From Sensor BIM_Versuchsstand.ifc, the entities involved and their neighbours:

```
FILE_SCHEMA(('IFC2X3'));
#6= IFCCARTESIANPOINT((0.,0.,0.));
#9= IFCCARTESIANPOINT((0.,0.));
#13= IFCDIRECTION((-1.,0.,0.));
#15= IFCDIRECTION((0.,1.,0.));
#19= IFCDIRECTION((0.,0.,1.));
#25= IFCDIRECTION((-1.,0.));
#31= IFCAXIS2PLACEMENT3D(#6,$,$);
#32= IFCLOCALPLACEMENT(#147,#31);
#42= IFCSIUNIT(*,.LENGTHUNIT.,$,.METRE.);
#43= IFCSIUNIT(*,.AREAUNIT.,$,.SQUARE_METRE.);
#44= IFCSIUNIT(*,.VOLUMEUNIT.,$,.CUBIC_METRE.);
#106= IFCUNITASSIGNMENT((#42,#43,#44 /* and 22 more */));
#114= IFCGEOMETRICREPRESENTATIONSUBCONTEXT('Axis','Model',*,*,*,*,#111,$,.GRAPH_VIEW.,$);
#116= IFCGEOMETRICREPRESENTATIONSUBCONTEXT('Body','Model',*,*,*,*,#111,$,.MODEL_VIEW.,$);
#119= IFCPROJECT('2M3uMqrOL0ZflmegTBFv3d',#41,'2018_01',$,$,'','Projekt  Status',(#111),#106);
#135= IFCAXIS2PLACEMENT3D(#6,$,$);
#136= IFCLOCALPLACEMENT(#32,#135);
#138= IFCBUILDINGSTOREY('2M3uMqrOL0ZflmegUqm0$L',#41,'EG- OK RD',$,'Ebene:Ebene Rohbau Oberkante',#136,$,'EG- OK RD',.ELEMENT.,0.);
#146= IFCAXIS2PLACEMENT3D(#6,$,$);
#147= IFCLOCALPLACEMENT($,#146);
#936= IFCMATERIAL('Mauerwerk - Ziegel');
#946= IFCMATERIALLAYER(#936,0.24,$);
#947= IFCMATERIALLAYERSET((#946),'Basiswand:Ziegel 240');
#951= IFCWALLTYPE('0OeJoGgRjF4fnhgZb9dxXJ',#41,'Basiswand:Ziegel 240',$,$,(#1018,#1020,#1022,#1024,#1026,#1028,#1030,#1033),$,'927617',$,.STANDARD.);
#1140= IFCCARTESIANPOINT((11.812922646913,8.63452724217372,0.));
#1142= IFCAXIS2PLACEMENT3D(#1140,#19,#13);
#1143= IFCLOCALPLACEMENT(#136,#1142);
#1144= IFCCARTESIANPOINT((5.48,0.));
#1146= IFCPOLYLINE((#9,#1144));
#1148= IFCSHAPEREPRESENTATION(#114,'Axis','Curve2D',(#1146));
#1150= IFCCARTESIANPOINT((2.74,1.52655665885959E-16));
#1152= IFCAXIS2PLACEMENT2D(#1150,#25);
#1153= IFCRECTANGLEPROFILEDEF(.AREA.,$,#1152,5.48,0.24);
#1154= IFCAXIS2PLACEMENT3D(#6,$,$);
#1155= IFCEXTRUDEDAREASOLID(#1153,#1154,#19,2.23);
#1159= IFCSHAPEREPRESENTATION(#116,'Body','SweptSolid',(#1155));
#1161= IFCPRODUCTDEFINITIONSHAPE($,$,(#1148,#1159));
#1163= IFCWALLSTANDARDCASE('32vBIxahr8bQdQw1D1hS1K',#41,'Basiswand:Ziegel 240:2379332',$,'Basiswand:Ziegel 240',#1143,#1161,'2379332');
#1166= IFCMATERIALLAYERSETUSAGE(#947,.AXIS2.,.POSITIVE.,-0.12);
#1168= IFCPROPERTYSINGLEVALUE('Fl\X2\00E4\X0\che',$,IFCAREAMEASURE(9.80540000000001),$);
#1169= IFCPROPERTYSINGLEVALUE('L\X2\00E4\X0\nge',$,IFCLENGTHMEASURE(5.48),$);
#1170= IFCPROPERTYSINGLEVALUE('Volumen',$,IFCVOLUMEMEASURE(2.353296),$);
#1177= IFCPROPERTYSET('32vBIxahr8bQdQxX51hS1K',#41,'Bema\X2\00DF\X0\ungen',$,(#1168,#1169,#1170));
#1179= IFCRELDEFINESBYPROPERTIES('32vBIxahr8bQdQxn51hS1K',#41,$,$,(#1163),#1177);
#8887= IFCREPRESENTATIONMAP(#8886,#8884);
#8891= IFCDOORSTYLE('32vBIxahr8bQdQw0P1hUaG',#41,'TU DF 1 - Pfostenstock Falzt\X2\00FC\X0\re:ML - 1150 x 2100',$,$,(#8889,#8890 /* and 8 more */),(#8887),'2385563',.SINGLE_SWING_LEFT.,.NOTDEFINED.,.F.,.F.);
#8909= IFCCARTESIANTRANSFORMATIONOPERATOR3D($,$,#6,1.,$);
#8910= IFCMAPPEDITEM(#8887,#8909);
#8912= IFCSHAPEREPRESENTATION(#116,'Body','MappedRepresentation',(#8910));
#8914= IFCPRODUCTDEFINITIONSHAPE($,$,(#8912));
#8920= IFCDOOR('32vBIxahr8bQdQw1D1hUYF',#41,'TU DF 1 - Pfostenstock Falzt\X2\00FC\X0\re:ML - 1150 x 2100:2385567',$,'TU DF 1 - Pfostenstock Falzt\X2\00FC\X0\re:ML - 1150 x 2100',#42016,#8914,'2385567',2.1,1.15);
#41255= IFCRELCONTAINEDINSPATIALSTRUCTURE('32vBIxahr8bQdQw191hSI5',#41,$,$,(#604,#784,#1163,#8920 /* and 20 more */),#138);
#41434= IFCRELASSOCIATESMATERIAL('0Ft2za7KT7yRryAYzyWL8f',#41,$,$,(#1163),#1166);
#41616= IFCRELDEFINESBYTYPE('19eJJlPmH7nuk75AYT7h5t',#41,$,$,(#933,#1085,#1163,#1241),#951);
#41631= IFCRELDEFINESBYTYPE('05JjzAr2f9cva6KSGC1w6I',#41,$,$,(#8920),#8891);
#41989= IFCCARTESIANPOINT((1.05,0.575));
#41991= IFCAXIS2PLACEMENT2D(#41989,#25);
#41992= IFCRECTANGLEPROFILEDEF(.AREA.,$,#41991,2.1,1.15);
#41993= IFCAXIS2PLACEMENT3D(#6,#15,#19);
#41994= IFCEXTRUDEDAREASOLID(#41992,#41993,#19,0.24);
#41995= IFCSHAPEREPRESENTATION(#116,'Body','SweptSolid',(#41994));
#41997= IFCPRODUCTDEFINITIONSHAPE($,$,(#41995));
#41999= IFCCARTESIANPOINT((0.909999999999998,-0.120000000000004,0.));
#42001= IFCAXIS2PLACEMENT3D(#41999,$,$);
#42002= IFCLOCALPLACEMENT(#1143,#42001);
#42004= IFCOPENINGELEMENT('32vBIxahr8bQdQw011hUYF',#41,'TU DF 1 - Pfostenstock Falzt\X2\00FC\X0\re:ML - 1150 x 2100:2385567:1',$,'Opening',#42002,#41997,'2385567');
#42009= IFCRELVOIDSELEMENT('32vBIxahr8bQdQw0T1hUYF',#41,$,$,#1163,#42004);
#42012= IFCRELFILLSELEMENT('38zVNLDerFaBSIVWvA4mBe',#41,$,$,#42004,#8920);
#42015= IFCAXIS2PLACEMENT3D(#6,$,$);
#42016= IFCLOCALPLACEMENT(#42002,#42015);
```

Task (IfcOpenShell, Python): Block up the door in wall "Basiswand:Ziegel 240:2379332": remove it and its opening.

```python
import ifcopenshell
import ifcopenshell.api.feature
import ifcopenshell.api.pset
import ifcopenshell.api.root
import ifcopenshell.geom
import ifcopenshell.util.element
import ifcopenshell.util.shape
import ifcopenshell.util.unit

model = ifcopenshell.open("Sensor BIM_Versuchsstand.ifc")
area_scale = ifcopenshell.util.unit.calculate_unit_scale(model, "AREAUNIT")
volume_scale = ifcopenshell.util.unit.calculate_unit_scale(model, "VOLUMEUNIT")
settings = ifcopenshell.geom.settings()


def volume(element):
    """Net volume in cubic metres, openings subtracted."""
    shape = ifcopenshell.geom.create_shape(settings, element)
    return ifcopenshell.util.shape.get_volume(shape.geometry)


door = model.by_guid("32vBIxahr8bQdQw1D1hUYF")
opening = door.FillsVoids[0].RelatingOpeningElement
wall = opening.VoidsElements[0].RelatingBuildingElement
before = volume(wall)

ifcopenshell.api.root.remove_product(model, product=door)
ifcopenshell.api.feature.remove_feature(model, feature=opening)

after = volume(wall)
thickness = 0.24  # wall thickness in metres

# Update the wall's stored quantities.
pset = model.by_id(ifcopenshell.util.element.get_pset(wall, "Bemaßungen", should_inherit=False)["id"])
ifcopenshell.api.pset.edit_pset(model, pset=pset, properties={
    "Fläche": model.create_entity("IfcAreaMeasure", after / thickness / area_scale),
    "Volumen": model.create_entity("IfcVolumeMeasure", after / volume_scale),
})

print(f"wall volume {before:.3f} -> {after:.3f} m3")

model.write("Sensor BIM_Versuchsstand_v2.ifc")
```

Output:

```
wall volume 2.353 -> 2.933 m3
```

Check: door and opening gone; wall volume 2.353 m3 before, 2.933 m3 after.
